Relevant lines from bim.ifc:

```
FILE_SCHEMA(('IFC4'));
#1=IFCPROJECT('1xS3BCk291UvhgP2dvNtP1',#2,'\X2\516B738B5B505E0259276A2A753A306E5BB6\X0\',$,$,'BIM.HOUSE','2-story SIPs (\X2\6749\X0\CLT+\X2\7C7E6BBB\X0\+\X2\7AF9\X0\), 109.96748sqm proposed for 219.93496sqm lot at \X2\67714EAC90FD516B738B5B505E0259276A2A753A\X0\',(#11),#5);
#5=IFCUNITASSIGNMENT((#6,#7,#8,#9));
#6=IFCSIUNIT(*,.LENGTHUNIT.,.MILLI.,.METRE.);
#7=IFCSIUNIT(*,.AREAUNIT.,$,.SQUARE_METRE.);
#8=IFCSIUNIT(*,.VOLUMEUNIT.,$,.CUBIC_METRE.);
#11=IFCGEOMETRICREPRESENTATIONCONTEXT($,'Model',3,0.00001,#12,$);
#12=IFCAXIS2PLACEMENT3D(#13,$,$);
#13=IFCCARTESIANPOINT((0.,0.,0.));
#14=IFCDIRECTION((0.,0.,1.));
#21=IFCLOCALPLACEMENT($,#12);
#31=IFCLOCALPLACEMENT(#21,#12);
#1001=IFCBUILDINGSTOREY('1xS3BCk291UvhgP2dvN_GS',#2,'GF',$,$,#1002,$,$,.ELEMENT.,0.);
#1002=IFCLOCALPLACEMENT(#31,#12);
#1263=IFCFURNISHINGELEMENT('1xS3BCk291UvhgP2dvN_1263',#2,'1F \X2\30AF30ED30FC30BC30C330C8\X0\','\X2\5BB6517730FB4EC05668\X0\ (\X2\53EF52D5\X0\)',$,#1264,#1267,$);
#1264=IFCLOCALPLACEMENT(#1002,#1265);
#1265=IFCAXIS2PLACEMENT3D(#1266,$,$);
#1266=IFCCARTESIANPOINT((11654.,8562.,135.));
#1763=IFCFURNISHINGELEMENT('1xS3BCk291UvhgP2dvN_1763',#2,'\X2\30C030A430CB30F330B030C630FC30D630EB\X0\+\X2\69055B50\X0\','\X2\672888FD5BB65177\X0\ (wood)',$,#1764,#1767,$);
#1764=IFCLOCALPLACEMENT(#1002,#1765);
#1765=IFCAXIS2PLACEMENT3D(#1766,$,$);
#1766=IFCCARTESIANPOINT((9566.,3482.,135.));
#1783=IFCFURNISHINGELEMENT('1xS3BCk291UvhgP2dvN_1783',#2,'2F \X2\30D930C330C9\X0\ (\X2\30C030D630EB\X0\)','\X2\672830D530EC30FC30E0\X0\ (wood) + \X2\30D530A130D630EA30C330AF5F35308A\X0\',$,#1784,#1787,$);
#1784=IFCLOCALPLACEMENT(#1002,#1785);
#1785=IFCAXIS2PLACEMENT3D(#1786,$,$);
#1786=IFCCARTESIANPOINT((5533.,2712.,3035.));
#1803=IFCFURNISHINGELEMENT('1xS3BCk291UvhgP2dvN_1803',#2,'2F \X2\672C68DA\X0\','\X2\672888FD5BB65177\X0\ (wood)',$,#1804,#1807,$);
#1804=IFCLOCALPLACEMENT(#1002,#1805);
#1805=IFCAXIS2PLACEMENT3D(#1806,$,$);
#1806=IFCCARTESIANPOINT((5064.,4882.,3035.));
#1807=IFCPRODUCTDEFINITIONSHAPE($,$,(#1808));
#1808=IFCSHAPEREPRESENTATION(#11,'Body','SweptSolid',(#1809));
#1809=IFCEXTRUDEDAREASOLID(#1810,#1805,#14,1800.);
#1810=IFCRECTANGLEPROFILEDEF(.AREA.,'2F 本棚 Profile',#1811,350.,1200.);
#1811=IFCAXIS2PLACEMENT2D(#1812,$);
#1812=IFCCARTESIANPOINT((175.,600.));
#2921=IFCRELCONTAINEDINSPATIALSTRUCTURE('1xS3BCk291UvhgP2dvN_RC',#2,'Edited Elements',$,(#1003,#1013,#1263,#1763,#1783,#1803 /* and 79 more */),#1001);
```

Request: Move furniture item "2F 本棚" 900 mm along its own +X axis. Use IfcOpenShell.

```python
import ifcopenshell
import ifcopenshell.api.geometry
import ifcopenshell.util.placement
import ifcopenshell.util.unit

model = ifcopenshell.open("bim.ifc")
unit_scale = ifcopenshell.util.unit.calculate_unit_scale(model)

item = model.by_id(1803)
matrix = ifcopenshell.util.placement.get_local_placement(item.ObjectPlacement)
matrix[:3, 3] += matrix[:3, 0] * 0.9 / unit_scale
ifcopenshell.api.geometry.edit_object_placement(model, product=item, matrix=matrix, is_si=False)

print(ifcopenshell.util.placement.get_local_placement(item.ObjectPlacement).round(3) + 0.0)

model.write("bim_v2.ifc")
```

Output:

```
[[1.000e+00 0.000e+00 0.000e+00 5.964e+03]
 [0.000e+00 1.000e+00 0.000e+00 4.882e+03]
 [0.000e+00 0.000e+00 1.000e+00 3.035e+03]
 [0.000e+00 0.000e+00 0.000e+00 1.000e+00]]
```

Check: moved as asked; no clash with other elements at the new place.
